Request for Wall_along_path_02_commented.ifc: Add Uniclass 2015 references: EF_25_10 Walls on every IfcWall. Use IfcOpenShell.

First a look at what the model holds.

```python
import ifcopenshell

model = ifcopenshell.open("Wall_along_path_02_commented.ifc")
print(model.schema)
print("classifications:", [c.Name for c in model.by_type("IfcClassification")])
for ifc_class in ("IfcDoor", "IfcRoof", "IfcStair", "IfcWall", "IfcWindow"):
    print(ifc_class, len(model.by_type(ifc_class)))
```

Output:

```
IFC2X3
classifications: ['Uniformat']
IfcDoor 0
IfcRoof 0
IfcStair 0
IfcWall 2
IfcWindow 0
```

```python
import ifcopenshell
import ifcopenshell.api.classification

model = ifcopenshell.open("Wall_along_path_02_commented.ifc")

# IFC2X3 requires Source and Edition and has no link from the project to the system.
system = model.create_entity("IfcClassification", Source="NBS", Edition="2015", Name="Uniclass 2015")

codes = {
    "IfcWall": ("EF_25_10", "Walls"),
}
for ifc_class, (code, name) in codes.items():
    products = model.by_type(ifc_class)
    ifcopenshell.api.classification.add_reference(
        model, products=products, classification=system, identification=code, name=name
    )
    print(code, len(products))

model.write("Wall_along_path_02_commented-out.ifc")
```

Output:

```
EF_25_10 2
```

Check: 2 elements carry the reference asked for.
